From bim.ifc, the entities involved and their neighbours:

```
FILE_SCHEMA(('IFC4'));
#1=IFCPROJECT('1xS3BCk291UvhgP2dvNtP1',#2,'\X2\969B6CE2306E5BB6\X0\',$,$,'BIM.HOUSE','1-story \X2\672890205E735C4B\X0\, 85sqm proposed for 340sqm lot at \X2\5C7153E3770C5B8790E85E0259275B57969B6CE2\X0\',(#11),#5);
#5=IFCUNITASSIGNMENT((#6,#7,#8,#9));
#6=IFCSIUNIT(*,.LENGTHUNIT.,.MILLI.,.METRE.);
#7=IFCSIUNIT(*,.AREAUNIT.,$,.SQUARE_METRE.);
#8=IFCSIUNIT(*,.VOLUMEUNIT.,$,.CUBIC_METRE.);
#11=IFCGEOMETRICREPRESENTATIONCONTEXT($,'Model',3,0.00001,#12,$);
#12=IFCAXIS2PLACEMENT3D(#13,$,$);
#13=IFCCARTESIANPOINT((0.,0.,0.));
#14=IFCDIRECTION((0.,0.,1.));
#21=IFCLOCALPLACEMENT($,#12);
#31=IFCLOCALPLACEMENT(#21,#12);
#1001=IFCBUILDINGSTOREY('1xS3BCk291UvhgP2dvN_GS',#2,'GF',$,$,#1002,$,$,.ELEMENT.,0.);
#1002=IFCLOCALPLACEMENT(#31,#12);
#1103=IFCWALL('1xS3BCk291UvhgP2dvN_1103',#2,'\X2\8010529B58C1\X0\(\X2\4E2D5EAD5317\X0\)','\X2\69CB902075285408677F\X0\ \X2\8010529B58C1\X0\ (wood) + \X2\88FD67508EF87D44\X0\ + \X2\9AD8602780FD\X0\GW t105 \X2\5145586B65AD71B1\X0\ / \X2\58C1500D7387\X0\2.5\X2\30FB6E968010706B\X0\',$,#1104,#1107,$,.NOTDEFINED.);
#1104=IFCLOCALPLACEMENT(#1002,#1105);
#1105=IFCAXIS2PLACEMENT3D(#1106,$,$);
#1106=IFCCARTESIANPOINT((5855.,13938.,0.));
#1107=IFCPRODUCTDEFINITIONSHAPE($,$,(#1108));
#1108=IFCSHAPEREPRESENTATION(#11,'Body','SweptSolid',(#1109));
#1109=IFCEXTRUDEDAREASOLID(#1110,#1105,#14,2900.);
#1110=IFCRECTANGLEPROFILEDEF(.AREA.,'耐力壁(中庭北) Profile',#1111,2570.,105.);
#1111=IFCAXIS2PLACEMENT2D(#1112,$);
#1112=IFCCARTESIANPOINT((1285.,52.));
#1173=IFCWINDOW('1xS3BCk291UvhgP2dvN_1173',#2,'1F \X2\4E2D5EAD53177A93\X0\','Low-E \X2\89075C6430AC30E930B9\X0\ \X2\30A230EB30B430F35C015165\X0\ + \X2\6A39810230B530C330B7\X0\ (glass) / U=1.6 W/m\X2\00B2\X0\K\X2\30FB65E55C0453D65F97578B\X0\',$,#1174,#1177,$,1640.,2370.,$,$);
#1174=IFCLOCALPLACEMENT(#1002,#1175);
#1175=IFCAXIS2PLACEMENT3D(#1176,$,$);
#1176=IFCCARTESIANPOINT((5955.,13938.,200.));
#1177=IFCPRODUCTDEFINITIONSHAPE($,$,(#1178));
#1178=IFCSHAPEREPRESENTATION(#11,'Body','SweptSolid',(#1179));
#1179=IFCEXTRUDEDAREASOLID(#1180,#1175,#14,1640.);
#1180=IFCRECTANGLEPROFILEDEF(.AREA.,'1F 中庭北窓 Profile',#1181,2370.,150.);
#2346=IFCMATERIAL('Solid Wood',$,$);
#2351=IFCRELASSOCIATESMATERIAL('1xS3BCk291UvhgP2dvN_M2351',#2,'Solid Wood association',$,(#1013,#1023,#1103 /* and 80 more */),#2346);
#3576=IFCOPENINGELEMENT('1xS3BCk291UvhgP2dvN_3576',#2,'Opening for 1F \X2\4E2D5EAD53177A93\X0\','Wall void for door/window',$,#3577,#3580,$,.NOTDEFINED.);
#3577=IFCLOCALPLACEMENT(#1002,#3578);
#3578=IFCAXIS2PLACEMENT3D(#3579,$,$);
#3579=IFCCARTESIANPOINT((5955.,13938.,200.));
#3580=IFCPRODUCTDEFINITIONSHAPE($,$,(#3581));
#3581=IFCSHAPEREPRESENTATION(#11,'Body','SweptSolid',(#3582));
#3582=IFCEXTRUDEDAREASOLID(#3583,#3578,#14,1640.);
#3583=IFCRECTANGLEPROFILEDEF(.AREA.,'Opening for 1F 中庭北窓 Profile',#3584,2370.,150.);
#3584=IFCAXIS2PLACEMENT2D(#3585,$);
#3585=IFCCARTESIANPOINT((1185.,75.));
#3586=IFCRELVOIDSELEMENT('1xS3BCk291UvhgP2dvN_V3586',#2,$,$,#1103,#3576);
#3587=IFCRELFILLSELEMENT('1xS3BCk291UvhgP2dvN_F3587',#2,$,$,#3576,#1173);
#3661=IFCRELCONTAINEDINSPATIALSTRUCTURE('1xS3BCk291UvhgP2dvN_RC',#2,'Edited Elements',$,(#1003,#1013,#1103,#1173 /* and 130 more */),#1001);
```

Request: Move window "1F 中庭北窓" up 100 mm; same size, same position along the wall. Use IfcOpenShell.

```python
import numpy as np
import ifcopenshell
import ifcopenshell.api.geometry
import ifcopenshell.util.placement
import ifcopenshell.util.unit

model = ifcopenshell.open("bim.ifc")
unit_scale = ifcopenshell.util.unit.calculate_unit_scale(model)

window = model.by_guid("1xS3BCk291UvhgP2dvN_1173")
opening = window.FillsVoids[0].RelatingOpeningElement
dz = 0.1 / unit_scale

shift = np.array([0.0, 0.0, dz])
# The window is not placed relative to its opening, so move both.
for product in (opening, window):
    matrix = ifcopenshell.util.placement.get_local_placement(product.ObjectPlacement)
    matrix[:3, 3] += shift
    ifcopenshell.api.geometry.edit_object_placement(model, product=product, matrix=matrix, is_si=False)

print(f"moved by {dz * unit_scale:+.3f} m")

model.write("bim_updated.ifc")
```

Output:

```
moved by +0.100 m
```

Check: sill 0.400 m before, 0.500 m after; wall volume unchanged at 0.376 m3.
